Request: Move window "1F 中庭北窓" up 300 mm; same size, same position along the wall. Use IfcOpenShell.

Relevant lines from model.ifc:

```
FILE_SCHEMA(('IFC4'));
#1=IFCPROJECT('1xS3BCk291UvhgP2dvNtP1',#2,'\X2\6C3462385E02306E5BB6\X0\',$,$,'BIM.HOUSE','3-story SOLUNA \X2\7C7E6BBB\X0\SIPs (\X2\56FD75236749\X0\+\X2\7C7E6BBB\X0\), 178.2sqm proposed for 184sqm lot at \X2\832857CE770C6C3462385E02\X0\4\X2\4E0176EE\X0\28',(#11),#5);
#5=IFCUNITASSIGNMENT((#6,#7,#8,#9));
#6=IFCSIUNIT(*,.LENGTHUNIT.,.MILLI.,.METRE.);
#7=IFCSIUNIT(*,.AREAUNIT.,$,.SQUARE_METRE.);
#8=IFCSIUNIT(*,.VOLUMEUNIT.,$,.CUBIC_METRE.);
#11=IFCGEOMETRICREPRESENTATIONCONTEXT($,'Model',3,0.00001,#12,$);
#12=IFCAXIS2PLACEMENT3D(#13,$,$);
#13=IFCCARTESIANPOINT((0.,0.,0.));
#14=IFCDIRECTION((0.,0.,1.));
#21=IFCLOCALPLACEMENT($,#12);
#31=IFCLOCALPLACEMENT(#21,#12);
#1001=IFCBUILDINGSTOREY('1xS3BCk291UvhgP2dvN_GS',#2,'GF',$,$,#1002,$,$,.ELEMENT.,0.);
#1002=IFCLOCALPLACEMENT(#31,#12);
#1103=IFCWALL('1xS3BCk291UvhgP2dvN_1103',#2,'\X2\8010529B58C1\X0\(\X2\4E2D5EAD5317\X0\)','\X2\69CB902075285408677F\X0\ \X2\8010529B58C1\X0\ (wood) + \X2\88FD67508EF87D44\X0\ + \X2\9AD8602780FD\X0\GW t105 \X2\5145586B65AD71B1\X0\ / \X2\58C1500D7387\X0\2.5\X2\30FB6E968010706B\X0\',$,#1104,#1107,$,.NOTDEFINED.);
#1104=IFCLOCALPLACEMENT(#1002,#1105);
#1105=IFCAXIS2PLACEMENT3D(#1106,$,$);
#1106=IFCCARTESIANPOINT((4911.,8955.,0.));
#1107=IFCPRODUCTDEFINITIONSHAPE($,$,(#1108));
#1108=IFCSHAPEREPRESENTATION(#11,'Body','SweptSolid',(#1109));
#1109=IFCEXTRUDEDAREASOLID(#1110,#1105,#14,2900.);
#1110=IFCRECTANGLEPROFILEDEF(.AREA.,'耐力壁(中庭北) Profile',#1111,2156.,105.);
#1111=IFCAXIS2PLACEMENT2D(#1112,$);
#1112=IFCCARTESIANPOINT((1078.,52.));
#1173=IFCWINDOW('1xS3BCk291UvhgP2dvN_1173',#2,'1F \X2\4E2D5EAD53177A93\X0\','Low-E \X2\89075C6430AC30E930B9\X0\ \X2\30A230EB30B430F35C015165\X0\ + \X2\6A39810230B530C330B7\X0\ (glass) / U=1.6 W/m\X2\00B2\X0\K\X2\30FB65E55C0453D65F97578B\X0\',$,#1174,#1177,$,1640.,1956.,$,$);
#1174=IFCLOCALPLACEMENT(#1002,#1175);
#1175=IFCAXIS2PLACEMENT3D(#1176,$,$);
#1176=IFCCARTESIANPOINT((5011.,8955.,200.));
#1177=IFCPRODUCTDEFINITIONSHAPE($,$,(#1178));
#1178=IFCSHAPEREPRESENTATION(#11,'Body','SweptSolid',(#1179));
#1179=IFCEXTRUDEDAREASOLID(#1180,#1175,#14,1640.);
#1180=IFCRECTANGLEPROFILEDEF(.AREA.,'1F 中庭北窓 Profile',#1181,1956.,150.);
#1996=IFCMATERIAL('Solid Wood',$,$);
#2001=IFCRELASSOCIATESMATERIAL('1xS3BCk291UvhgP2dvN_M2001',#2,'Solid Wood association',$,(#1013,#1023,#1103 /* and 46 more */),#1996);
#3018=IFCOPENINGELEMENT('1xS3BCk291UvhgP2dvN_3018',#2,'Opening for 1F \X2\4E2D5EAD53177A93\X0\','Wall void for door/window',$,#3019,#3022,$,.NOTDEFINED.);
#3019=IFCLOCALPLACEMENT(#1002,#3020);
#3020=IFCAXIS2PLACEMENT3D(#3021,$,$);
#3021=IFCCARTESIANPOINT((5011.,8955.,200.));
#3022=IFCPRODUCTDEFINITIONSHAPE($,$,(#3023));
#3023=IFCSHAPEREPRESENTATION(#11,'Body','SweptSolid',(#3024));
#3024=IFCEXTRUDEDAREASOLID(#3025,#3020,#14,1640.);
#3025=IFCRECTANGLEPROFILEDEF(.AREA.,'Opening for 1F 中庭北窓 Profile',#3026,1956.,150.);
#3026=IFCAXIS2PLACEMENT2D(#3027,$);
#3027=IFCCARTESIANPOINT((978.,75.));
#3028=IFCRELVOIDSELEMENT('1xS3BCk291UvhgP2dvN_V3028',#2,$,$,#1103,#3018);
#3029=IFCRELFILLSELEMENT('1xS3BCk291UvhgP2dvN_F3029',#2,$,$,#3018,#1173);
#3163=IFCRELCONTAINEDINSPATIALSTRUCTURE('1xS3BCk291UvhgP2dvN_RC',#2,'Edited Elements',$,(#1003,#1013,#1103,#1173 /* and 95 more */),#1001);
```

```python
import numpy as np
import ifcopenshell
import ifcopenshell.api.geometry
import ifcopenshell.util.placement
import ifcopenshell.util.unit

model = ifcopenshell.open("model.ifc")
unit_scale = ifcopenshell.util.unit.calculate_unit_scale(model)

window = model.by_id(1173)
opening = window.FillsVoids[0].RelatingOpeningElement
dz = 300.0

shift = np.array([0.0, 0.0, dz])
# The window is not placed relative to its opening, so move both.
for product in (opening, window):
    matrix = ifcopenshell.util.placement.get_local_placement(product.ObjectPlacement)
    matrix[:3, 3] += shift
    ifcopenshell.api.geometry.edit_object_placement(model, product=product, matrix=matrix, is_si=False)

print(f"moved by {dz * unit_scale:+.3f} m")

model.write("model_edited.ifc")
```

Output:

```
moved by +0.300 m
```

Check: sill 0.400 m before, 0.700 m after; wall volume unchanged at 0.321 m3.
